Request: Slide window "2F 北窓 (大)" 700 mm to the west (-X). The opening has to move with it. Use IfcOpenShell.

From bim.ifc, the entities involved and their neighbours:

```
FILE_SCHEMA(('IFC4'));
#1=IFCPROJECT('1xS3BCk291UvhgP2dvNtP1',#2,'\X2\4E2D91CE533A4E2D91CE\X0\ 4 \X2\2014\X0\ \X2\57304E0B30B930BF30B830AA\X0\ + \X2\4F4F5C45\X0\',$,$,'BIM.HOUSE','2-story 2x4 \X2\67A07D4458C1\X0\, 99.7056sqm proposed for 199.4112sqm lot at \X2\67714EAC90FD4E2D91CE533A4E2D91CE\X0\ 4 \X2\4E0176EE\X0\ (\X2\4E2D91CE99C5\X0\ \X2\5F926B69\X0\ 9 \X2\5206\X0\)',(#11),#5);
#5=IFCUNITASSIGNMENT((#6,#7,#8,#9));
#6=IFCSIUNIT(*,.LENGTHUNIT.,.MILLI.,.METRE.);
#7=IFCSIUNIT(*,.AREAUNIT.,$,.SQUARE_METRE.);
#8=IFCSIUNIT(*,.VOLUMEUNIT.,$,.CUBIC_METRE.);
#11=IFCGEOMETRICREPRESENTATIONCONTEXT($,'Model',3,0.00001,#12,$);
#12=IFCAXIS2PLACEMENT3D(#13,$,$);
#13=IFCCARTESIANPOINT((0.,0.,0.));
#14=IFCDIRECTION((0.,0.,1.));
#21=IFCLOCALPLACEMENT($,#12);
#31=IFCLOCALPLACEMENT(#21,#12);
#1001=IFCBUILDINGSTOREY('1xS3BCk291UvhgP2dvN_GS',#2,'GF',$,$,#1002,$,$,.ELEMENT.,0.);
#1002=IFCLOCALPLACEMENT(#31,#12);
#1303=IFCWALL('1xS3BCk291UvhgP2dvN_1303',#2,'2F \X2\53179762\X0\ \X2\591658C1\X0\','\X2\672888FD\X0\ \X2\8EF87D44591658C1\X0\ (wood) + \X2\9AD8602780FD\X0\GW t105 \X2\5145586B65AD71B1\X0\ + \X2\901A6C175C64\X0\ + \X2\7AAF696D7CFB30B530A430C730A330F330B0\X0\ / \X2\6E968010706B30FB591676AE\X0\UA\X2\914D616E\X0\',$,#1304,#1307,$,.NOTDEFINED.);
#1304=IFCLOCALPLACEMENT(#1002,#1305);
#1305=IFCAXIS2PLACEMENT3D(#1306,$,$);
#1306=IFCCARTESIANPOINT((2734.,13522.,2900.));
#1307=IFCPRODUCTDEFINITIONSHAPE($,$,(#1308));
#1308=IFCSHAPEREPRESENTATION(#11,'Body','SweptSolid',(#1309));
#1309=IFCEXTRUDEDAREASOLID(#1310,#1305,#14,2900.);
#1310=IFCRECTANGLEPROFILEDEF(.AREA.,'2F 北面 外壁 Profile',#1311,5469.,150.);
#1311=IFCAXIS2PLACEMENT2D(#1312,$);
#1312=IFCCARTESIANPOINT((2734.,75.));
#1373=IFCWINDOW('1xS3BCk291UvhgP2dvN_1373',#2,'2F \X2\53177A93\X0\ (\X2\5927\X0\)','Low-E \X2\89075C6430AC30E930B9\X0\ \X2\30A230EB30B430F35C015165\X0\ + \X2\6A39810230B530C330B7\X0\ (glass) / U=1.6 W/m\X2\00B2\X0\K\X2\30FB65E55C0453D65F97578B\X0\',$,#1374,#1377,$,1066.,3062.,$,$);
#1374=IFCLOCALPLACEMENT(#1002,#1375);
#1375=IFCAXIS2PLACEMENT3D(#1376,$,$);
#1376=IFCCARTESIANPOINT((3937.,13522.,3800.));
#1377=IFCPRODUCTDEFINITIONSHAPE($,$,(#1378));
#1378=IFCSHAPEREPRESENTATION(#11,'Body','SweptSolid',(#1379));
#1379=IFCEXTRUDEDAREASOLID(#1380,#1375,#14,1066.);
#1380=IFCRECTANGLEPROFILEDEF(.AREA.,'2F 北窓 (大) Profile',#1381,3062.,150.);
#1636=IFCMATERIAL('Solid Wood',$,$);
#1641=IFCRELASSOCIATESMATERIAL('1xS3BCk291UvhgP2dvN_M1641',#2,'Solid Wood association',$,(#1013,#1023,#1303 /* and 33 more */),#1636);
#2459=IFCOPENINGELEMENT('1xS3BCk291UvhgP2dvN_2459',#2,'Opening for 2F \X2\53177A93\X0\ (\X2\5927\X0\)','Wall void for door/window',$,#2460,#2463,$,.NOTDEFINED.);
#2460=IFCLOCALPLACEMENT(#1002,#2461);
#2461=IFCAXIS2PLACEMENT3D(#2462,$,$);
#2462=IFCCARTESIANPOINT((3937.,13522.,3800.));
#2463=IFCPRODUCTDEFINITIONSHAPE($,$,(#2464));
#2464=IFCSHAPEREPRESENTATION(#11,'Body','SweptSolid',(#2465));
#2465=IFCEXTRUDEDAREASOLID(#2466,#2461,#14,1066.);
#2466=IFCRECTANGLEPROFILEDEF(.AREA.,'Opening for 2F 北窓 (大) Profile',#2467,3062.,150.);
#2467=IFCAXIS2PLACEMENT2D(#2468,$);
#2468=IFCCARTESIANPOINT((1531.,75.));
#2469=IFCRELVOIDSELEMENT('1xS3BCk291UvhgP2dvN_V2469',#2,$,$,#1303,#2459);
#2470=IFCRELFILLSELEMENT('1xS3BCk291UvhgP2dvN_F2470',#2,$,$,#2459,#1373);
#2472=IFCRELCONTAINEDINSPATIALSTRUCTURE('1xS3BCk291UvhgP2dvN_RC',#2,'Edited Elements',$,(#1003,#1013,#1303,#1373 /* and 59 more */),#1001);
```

```python
import ifcopenshell
import ifcopenshell.api.geometry
import ifcopenshell.util.placement
import ifcopenshell.util.unit

model = ifcopenshell.open("bim.ifc")
unit_scale = ifcopenshell.util.unit.calculate_unit_scale(model)

window = model.by_guid("1xS3BCk291UvhgP2dvN_1373")
opening = window.FillsVoids[0].RelatingOpeningElement
wall = opening.VoidsElements[0].RelatingBuildingElement

wall_matrix = ifcopenshell.util.placement.get_local_placement(wall.ObjectPlacement)
shift = wall_matrix[:3, 0] * -0.7 / unit_scale
before = ifcopenshell.util.placement.get_local_placement(window.ObjectPlacement)[:3, 3].copy()

# The window is not placed relative to its opening, so move both.
for product in (opening, window):
    matrix = ifcopenshell.util.placement.get_local_placement(product.ObjectPlacement)
    matrix[:3, 3] += shift
    ifcopenshell.api.geometry.edit_object_placement(model, product=product, matrix=matrix, is_si=False)

after = ifcopenshell.util.placement.get_local_placement(window.ObjectPlacement)[:3, 3]
print("window moved by", (after - before).round(3) + 0.0)

model.write("bim_updated.ifc")
```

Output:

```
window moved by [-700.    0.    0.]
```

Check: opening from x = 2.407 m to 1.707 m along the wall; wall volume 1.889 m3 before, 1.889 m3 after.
